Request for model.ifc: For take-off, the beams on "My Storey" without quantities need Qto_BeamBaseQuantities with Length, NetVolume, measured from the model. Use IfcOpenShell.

First a look at what the model holds.

```python
import ifcopenshell
import ifcopenshell.util.element
import ifcopenshell.util.unit

model = ifcopenshell.open("model.ifc")
print(model.schema)
for unit_type in ("LENGTHUNIT", "AREAUNIT", "VOLUMEUNIT"):
    print(unit_type, ifcopenshell.util.unit.calculate_unit_scale(model, unit_type))
storey = next(s for s in model.by_type("IfcBuildingStorey") if s.Name == "My Storey")
beams = [e for e in ifcopenshell.util.element.get_decomposition(storey) if e.is_a("IfcBeam")]
for e in sorted(beams, key=lambda e: e.id()):
    print(e.id(), e.is_a(), e.Name, list(ifcopenshell.util.element.get_psets(e, qtos_only=True)), sep=" | ")
```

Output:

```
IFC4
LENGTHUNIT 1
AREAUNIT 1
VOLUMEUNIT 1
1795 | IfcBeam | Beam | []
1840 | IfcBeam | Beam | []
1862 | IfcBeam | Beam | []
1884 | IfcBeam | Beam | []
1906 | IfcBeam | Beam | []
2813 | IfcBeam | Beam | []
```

```python
import ifcopenshell
import ifcopenshell.api.pset
import ifcopenshell.geom
import ifcopenshell.util.element
import ifcopenshell.util.shape
import ifcopenshell.util.unit

model = ifcopenshell.open("model.ifc")
unit_scale = ifcopenshell.util.unit.calculate_unit_scale(model)
volume_scale = ifcopenshell.util.unit.calculate_unit_scale(model, "VOLUMEUNIT")
settings = ifcopenshell.geom.settings()

storey = next(s for s in model.by_type("IfcBuildingStorey") if s.Name == "My Storey")
beams = [e for e in ifcopenshell.util.element.get_decomposition(storey) if e.is_a("IfcBeam")]

for e in sorted(beams, key=lambda e: e.id()):
    if ifcopenshell.util.element.get_psets(e, qtos_only=True, should_inherit=False):
        continue
    # Geometry comes back in metres, in the element's own axes.
    shape = ifcopenshell.geom.create_shape(settings, e)
    values = {
        "Length": ifcopenshell.util.shape.get_max_xyz(shape.geometry) / unit_scale,
        "NetVolume": ifcopenshell.util.shape.get_volume(shape.geometry) / volume_scale,
    }
    qto = ifcopenshell.api.pset.add_qto(model, product=e, name="Qto_BeamBaseQuantities")
    ifcopenshell.api.pset.edit_qto(model, qto=qto, properties=values)
    print(e.id(), {k: round(v, 3) for k, v in values.items()})

model.write("model_updated.ifc")
```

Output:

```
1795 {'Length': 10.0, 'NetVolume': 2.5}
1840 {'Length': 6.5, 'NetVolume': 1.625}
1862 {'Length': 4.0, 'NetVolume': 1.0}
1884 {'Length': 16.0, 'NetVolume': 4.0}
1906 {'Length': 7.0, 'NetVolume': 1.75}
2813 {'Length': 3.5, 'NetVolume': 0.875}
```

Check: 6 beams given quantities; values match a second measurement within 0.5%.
